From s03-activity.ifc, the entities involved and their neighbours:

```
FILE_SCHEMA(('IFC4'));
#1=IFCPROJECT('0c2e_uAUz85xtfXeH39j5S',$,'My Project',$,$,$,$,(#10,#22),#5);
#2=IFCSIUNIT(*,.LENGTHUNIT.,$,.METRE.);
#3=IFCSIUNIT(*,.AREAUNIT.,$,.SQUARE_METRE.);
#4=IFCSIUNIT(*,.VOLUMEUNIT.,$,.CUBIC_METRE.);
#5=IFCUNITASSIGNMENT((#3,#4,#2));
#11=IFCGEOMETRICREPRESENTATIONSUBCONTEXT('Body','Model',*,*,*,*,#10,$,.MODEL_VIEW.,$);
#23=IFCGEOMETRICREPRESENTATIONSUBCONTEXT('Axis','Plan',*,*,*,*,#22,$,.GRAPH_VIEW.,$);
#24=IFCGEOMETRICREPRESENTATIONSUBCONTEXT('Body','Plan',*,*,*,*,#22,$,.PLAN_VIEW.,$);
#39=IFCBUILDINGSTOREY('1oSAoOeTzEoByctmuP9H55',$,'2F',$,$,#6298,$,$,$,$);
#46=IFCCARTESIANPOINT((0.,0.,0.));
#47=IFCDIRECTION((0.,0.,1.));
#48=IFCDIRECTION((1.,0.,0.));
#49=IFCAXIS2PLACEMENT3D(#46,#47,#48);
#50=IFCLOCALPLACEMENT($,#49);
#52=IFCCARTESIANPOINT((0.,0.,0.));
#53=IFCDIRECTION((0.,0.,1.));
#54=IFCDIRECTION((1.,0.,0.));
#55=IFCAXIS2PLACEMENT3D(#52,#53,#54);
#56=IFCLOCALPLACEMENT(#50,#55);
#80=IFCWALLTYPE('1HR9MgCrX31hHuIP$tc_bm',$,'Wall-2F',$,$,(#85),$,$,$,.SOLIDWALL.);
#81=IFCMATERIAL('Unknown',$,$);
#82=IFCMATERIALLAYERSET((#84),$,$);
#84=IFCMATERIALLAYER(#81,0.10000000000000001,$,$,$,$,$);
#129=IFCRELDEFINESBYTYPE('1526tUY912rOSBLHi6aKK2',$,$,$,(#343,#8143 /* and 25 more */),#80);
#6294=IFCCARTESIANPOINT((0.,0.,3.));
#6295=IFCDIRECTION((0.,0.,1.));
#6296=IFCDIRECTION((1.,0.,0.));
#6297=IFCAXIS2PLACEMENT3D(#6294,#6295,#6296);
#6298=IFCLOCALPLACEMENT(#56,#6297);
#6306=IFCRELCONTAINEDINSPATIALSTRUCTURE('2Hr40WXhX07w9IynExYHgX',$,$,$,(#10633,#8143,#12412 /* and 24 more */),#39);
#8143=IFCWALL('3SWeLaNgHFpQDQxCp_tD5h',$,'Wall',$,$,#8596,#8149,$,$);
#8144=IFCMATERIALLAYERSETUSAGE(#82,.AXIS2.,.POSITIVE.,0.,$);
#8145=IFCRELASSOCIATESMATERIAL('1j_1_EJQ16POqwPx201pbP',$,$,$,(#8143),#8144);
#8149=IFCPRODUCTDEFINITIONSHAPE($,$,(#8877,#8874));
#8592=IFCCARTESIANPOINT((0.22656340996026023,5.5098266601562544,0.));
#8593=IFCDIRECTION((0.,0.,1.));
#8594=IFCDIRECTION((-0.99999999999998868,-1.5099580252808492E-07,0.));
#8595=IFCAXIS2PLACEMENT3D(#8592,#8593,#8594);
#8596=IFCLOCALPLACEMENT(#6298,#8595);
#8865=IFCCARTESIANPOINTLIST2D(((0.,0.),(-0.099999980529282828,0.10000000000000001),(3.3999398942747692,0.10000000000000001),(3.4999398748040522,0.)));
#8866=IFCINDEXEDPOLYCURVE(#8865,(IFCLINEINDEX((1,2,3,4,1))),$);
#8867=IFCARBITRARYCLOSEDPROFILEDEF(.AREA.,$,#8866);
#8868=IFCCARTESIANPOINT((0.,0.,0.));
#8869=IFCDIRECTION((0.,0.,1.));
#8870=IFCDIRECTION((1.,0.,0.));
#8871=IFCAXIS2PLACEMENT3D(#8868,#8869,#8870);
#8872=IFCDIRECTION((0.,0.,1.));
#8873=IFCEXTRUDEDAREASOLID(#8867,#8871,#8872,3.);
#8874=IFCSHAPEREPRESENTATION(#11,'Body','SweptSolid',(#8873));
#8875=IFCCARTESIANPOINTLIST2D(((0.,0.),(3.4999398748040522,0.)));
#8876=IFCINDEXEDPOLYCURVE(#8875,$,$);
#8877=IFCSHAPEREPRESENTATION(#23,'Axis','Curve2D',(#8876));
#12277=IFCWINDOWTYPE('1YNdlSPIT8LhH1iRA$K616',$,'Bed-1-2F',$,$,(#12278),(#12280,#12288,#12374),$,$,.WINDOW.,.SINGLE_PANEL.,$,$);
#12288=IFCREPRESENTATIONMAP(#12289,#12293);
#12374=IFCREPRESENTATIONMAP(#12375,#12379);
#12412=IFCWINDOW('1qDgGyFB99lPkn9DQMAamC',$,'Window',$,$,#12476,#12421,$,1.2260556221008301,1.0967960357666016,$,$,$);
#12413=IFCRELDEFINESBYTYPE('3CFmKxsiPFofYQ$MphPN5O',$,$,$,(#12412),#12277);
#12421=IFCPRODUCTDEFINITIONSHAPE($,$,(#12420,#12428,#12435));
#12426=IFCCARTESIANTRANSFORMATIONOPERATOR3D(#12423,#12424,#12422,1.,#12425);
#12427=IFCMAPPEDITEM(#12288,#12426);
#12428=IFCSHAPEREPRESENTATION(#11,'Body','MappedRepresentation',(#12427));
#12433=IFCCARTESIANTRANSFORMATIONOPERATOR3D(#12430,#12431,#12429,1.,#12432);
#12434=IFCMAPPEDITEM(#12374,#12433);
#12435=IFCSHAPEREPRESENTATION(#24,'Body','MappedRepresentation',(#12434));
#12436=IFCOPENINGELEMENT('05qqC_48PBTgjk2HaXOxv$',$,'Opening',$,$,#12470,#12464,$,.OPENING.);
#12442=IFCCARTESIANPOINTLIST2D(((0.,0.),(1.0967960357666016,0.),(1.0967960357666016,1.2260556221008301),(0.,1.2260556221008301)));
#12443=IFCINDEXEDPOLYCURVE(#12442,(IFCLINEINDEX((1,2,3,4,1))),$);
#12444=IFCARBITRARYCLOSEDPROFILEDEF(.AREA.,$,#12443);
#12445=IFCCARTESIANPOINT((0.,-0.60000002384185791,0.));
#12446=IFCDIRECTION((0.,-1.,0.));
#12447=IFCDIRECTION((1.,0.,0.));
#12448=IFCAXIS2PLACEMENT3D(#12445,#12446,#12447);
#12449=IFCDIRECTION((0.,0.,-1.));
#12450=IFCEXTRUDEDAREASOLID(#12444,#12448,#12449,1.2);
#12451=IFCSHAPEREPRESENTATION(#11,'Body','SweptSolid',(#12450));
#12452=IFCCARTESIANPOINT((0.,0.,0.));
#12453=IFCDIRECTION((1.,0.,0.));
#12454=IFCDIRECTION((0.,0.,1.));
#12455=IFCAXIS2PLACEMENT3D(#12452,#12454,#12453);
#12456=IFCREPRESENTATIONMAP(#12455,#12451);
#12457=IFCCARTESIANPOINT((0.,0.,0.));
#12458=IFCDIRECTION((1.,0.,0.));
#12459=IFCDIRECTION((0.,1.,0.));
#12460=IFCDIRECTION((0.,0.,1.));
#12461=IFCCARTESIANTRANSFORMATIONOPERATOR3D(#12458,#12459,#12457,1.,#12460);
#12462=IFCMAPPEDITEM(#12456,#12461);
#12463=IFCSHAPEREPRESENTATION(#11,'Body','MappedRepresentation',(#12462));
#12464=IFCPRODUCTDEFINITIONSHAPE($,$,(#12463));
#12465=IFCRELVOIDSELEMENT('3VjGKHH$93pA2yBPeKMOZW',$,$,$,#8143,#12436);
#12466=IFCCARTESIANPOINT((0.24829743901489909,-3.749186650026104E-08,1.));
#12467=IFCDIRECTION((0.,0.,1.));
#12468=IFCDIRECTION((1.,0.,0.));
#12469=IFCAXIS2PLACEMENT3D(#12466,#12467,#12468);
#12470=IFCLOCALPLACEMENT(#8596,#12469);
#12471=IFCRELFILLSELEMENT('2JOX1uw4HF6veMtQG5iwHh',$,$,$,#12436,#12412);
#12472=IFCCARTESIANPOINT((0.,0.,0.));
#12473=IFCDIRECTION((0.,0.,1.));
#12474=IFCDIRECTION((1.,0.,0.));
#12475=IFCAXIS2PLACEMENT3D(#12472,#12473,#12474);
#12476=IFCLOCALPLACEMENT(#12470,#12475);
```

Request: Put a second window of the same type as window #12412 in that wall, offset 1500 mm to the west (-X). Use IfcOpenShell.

```python
import ifcopenshell
import ifcopenshell.api.feature
import ifcopenshell.api.geometry
import ifcopenshell.api.root
import ifcopenshell.geom
import ifcopenshell.util.element
import ifcopenshell.util.placement
import ifcopenshell.util.shape

model = ifcopenshell.open("s03-activity.ifc")
settings = ifcopenshell.geom.settings()


def volume(element):
    """Net volume in cubic metres, openings subtracted."""
    shape = ifcopenshell.geom.create_shape(settings, element)
    return ifcopenshell.util.shape.get_volume(shape.geometry)


window = model.by_id(12412)
opening = window.FillsVoids[0].RelatingOpeningElement
wall = opening.VoidsElements[0].RelatingBuildingElement
before = volume(wall)
shift = ifcopenshell.util.placement.get_local_placement(wall.ObjectPlacement)[:3, 0] * 1.5

# copy_class copies the void relationship, type, container and properties, but no geometry.
new_opening = ifcopenshell.api.root.copy_class(model, product=opening)
new_opening.Representation = ifcopenshell.util.element.copy_deep(
    model, opening.Representation, exclude=["IfcGeometricRepresentationContext", "IfcRepresentationMap"]
)
new_window = ifcopenshell.api.root.copy_class(model, product=window)
new_window.Representation = ifcopenshell.util.element.copy_deep(
    model, window.Representation, exclude=["IfcGeometricRepresentationContext", "IfcRepresentationMap"]
)
ifcopenshell.api.feature.add_filling(model, opening=new_opening, element=new_window)

for old, new in ((opening, new_opening), (window, new_window)):
    matrix = ifcopenshell.util.placement.get_local_placement(old.ObjectPlacement)
    matrix[:3, 3] += shift
    ifcopenshell.api.geometry.edit_object_placement(model, product=new, matrix=matrix, is_si=False)

after = volume(wall)

print(f"wall volume {before:.3f} -> {after:.3f} m3")

model.write("s03-activity_v2.ifc")
```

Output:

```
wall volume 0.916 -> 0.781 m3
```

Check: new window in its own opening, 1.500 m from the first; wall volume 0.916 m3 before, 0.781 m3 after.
